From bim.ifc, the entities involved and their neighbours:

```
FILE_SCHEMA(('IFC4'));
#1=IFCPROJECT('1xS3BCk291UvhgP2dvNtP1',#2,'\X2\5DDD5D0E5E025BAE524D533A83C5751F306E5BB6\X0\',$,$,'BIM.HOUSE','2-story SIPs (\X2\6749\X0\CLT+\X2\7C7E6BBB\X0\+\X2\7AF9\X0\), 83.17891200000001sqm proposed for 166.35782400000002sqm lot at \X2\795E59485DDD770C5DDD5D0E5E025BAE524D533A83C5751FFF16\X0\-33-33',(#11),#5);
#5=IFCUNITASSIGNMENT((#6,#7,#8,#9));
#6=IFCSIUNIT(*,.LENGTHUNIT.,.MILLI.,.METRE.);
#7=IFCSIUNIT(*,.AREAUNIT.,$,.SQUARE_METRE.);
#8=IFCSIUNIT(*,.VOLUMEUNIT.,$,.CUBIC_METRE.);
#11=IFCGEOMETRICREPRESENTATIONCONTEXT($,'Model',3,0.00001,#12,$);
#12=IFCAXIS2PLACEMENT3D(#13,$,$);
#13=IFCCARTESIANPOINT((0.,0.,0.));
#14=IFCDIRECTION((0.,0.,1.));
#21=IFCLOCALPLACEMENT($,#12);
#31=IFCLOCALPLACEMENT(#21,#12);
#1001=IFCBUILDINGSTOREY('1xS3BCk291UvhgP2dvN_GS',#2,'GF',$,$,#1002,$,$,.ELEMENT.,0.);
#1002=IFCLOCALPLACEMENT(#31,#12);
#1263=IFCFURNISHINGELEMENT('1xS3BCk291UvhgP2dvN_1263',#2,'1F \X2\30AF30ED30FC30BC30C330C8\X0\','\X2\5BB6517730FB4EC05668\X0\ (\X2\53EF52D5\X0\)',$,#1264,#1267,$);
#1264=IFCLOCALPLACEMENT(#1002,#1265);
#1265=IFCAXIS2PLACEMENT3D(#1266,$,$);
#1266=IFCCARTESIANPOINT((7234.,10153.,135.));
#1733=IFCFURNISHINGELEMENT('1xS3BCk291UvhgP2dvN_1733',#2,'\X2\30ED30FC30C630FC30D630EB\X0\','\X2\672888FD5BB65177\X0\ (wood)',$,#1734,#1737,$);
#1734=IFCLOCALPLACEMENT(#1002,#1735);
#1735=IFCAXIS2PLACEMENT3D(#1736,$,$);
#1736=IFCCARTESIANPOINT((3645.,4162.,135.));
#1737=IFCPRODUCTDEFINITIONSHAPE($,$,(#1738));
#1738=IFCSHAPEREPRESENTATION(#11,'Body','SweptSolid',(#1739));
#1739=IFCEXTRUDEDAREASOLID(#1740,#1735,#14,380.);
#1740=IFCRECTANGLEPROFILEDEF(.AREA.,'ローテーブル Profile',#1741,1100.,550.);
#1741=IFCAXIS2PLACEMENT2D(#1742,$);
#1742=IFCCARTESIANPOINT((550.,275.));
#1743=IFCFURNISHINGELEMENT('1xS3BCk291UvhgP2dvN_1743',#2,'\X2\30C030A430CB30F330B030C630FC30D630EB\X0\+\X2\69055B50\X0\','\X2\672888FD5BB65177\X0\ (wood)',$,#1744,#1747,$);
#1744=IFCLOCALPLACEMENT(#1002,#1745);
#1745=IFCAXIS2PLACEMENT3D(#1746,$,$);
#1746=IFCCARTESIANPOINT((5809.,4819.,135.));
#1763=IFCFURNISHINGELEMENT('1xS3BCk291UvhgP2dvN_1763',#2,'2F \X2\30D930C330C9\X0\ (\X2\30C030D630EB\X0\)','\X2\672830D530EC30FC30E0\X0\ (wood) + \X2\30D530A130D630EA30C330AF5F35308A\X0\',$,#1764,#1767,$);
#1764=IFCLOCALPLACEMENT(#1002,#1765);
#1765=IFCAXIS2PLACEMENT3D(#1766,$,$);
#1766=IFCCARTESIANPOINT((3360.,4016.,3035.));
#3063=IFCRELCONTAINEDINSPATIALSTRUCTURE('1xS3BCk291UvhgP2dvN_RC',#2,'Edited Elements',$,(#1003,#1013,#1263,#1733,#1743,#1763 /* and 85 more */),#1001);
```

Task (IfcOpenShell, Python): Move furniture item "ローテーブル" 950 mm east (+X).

```python
import ifcopenshell
import ifcopenshell.api.geometry
import ifcopenshell.util.placement

model = ifcopenshell.open("bim.ifc")

item = model.by_guid("1xS3BCk291UvhgP2dvN_1733")
matrix = ifcopenshell.util.placement.get_local_placement(item.ObjectPlacement)
matrix[0, 3] += 950.0
ifcopenshell.api.geometry.edit_object_placement(model, product=item, matrix=matrix, is_si=False)

print(ifcopenshell.util.placement.get_local_placement(item.ObjectPlacement).round(3) + 0.0)

model.write("bim-out.ifc")
```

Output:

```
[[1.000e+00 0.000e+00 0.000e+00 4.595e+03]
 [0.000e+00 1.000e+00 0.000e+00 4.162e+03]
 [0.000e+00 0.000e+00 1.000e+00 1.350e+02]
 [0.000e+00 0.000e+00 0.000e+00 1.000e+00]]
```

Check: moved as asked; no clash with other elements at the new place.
